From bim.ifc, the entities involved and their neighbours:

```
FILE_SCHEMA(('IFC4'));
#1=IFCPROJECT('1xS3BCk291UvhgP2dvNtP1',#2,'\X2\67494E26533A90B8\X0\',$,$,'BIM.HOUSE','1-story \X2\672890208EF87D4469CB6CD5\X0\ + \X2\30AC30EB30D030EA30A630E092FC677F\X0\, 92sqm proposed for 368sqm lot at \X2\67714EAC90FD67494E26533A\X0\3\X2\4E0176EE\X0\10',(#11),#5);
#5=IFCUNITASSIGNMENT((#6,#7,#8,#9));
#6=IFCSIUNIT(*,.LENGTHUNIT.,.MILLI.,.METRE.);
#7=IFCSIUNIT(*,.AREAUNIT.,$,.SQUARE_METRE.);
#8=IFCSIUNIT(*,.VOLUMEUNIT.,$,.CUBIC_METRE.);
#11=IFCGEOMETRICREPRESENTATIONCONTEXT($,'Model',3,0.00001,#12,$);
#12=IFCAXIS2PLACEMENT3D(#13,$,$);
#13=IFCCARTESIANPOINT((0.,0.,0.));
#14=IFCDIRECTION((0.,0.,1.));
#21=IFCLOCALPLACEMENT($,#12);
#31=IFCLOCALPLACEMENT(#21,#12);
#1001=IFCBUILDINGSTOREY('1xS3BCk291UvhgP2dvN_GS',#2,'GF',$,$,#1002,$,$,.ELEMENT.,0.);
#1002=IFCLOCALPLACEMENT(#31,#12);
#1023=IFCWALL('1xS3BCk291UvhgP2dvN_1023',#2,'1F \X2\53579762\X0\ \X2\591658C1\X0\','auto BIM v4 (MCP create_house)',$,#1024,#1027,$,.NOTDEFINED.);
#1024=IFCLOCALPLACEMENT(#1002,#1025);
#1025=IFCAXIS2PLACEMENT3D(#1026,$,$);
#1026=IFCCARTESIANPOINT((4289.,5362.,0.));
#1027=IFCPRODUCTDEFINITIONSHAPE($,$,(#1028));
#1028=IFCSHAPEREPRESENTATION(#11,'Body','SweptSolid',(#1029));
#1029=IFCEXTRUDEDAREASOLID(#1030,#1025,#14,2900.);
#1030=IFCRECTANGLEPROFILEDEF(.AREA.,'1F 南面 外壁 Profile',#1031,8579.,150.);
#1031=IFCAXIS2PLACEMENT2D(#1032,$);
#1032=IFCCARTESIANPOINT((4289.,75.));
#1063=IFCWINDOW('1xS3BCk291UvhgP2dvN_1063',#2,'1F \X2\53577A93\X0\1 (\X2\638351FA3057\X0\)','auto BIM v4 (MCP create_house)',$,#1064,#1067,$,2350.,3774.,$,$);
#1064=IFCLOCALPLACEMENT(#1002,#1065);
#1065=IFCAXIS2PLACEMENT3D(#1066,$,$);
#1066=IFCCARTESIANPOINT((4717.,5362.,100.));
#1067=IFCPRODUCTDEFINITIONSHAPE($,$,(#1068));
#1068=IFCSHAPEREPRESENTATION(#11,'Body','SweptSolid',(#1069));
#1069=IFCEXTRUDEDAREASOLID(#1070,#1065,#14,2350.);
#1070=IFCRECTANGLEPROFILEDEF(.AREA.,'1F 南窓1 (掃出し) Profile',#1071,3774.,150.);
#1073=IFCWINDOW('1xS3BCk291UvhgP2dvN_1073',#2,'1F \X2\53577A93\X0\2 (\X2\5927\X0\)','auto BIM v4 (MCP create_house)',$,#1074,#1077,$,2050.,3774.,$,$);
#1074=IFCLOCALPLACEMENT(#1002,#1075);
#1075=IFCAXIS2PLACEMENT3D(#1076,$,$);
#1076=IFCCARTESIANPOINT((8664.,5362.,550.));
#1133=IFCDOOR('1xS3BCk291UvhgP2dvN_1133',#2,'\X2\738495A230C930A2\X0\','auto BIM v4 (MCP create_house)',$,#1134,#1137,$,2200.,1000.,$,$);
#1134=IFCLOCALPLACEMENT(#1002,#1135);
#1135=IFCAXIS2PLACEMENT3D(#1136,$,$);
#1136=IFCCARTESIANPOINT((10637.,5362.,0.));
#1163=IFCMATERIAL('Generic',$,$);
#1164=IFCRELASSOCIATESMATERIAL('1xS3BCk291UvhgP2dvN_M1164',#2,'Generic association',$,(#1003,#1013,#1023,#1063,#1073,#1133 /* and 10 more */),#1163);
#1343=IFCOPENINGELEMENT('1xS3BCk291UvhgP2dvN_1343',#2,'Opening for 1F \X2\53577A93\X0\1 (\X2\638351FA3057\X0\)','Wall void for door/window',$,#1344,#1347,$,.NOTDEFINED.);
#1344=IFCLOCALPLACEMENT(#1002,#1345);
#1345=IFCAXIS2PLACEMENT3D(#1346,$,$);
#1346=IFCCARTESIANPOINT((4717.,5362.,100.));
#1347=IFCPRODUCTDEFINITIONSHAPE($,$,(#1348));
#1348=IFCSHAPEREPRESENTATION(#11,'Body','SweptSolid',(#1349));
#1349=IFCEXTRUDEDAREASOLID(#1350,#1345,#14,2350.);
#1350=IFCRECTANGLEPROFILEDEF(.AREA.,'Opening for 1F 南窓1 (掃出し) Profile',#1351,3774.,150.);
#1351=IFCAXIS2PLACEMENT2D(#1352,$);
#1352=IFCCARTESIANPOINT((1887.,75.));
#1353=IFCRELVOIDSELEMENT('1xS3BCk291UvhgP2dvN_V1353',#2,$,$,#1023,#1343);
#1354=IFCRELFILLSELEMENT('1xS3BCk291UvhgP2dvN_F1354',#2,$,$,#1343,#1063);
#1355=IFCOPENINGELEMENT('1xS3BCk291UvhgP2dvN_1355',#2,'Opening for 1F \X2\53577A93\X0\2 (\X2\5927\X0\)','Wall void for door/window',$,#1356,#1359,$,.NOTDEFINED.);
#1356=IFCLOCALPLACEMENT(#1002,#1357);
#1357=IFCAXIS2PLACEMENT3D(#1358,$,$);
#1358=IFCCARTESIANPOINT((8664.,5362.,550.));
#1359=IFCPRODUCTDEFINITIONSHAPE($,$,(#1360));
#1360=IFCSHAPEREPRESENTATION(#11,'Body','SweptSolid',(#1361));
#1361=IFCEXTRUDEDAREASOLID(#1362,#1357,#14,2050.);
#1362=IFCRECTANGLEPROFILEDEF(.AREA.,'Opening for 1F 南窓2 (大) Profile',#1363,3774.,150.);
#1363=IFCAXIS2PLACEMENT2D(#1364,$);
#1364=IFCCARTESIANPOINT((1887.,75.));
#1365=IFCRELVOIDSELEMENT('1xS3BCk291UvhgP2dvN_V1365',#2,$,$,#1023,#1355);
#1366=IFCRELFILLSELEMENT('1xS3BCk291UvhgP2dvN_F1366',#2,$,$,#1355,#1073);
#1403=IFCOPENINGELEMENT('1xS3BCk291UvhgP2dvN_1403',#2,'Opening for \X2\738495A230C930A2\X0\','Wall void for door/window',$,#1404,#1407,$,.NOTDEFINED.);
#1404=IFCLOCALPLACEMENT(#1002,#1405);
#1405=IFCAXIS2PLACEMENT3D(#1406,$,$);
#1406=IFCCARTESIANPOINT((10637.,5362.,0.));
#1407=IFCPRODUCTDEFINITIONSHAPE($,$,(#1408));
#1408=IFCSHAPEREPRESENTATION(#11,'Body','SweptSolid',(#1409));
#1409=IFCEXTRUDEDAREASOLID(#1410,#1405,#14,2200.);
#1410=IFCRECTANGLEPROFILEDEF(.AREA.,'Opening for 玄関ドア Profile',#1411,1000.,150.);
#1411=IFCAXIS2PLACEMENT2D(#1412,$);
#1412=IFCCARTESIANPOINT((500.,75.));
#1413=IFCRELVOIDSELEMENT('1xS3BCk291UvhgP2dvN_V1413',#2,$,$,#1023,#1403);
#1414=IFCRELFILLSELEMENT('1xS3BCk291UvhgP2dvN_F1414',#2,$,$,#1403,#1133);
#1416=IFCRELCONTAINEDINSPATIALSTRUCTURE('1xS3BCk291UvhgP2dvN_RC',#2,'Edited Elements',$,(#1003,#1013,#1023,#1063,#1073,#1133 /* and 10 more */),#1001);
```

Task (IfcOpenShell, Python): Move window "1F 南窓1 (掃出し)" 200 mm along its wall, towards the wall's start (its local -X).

```python
import ifcopenshell
import ifcopenshell.api.geometry
import ifcopenshell.util.placement

model = ifcopenshell.open("bim.ifc")

window = model.by_guid("1xS3BCk291UvhgP2dvN_1063")
opening = window.FillsVoids[0].RelatingOpeningElement
wall = opening.VoidsElements[0].RelatingBuildingElement

wall_matrix = ifcopenshell.util.placement.get_local_placement(wall.ObjectPlacement)
shift = wall_matrix[:3, 0] * -200.0
before = ifcopenshell.util.placement.get_local_placement(window.ObjectPlacement)[:3, 3].copy()

# The window is not placed relative to its opening, so move both.
for product in (opening, window):
    matrix = ifcopenshell.util.placement.get_local_placement(product.ObjectPlacement)
    matrix[:3, 3] += shift
    ifcopenshell.api.geometry.edit_object_placement(model, product=product, matrix=matrix, is_si=False)

after = ifcopenshell.util.placement.get_local_placement(window.ObjectPlacement)[:3, 3]
print("window moved by", (after - before).round(3) + 0.0)

model.write("bim_updated.ifc")
```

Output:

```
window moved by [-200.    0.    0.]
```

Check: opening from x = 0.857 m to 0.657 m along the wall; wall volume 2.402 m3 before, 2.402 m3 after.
